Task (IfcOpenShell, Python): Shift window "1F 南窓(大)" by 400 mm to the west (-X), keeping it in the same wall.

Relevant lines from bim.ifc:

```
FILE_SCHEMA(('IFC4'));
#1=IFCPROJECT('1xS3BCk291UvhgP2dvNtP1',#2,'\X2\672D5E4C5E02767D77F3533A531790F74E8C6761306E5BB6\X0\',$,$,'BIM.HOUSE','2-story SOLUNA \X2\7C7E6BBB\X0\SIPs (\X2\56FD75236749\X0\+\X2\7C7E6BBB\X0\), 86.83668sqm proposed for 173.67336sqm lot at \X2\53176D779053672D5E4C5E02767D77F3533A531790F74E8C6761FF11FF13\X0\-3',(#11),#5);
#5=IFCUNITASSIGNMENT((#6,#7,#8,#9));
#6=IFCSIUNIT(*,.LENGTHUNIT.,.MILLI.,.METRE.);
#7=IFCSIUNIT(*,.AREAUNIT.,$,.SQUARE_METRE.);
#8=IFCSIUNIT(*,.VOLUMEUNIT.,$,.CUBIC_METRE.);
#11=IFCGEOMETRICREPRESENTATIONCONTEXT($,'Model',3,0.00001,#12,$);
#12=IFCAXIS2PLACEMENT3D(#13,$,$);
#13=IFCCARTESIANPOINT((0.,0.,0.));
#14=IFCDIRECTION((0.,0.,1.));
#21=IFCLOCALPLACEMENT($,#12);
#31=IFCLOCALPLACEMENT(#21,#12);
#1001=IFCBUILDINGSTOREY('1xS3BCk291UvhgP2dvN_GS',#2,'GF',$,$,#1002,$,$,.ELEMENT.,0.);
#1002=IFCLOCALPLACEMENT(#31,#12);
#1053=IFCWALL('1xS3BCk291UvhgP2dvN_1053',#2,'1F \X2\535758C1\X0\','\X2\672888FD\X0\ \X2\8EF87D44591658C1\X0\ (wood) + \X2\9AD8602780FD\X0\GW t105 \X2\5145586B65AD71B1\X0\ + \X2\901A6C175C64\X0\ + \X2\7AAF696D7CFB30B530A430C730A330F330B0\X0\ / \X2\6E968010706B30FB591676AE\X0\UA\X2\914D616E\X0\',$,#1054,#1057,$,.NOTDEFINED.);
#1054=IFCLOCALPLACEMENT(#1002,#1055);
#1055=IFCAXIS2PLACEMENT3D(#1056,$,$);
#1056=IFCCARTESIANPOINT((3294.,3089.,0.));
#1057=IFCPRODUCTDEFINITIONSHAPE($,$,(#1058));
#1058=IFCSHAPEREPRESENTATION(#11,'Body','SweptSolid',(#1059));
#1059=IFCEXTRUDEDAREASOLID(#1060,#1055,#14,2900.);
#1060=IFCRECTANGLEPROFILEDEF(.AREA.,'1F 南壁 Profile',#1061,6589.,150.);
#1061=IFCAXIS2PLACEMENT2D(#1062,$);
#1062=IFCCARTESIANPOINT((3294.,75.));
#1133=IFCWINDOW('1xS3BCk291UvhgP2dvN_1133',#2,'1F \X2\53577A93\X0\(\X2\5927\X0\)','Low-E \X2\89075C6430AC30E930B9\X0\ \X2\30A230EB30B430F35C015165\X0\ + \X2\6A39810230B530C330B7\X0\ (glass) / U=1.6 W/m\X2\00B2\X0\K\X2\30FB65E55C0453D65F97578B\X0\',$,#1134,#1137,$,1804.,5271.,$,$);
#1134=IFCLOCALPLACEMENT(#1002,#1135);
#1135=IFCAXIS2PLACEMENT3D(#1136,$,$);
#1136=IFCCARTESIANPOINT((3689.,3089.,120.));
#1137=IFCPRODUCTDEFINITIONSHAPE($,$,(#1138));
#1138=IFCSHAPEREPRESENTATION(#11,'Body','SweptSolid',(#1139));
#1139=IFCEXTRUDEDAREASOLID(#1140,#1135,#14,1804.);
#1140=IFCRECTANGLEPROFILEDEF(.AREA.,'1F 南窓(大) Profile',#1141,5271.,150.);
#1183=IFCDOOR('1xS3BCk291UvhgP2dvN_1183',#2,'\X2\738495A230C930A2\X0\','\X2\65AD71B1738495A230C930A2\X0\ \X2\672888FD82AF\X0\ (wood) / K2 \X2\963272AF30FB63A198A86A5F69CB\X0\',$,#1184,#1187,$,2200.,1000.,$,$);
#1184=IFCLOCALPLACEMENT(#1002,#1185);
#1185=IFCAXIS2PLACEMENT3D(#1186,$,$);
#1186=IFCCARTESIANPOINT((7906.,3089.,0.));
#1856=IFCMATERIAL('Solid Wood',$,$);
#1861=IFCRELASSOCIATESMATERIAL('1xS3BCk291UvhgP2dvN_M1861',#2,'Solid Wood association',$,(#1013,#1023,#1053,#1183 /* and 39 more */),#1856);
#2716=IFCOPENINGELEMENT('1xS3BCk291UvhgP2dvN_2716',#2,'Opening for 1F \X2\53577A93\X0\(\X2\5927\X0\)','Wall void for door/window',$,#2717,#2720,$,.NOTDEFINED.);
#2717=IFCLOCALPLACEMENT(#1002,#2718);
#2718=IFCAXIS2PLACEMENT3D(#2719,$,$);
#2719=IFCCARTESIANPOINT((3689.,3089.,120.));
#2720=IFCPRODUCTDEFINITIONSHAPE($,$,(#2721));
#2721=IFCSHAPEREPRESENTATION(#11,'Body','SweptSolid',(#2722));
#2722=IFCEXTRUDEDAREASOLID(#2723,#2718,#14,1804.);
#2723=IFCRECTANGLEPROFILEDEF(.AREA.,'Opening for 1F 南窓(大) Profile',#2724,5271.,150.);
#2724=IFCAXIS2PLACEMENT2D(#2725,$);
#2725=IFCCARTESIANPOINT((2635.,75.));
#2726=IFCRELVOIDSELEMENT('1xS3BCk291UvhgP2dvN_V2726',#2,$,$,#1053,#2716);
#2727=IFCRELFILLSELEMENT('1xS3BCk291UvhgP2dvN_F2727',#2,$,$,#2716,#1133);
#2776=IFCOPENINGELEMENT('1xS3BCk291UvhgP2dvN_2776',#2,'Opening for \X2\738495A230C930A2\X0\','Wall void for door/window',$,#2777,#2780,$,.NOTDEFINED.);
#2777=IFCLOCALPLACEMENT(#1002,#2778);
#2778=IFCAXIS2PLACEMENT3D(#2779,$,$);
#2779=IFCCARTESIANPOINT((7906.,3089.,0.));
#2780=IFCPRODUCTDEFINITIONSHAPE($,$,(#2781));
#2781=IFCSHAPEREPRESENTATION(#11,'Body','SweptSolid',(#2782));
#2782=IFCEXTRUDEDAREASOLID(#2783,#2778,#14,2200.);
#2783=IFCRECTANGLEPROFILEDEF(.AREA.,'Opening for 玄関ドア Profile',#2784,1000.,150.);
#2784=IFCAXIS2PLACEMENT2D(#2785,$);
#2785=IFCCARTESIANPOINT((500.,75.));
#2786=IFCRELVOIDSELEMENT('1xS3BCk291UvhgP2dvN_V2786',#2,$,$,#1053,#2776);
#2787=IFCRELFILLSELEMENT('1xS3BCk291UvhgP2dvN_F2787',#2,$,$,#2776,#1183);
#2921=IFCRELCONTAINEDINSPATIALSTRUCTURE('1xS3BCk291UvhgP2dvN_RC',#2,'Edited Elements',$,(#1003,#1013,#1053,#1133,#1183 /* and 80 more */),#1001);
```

```python
import ifcopenshell
import ifcopenshell.api.geometry
import ifcopenshell.util.placement
import ifcopenshell.util.unit

model = ifcopenshell.open("bim.ifc")
unit_scale = ifcopenshell.util.unit.calculate_unit_scale(model)

window = model.by_guid("1xS3BCk291UvhgP2dvN_1133")
opening = window.FillsVoids[0].RelatingOpeningElement
wall = opening.VoidsElements[0].RelatingBuildingElement

wall_matrix = ifcopenshell.util.placement.get_local_placement(wall.ObjectPlacement)
shift = wall_matrix[:3, 0] * -0.4 / unit_scale
before = ifcopenshell.util.placement.get_local_placement(window.ObjectPlacement)[:3, 3].copy()

# The window is not placed relative to its opening, so move both.
for product in (opening, window):
    matrix = ifcopenshell.util.placement.get_local_placement(product.ObjectPlacement)
    matrix[:3, 3] += shift
    ifcopenshell.api.geometry.edit_object_placement(model, product=product, matrix=matrix, is_si=False)

after = ifcopenshell.util.placement.get_local_placement(window.ObjectPlacement)[:3, 3]
print("window moved by", (after - before).round(3) + 0.0)

model.write("bim_rev.ifc")
```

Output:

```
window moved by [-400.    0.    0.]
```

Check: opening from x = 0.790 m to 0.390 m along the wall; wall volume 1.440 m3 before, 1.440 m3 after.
